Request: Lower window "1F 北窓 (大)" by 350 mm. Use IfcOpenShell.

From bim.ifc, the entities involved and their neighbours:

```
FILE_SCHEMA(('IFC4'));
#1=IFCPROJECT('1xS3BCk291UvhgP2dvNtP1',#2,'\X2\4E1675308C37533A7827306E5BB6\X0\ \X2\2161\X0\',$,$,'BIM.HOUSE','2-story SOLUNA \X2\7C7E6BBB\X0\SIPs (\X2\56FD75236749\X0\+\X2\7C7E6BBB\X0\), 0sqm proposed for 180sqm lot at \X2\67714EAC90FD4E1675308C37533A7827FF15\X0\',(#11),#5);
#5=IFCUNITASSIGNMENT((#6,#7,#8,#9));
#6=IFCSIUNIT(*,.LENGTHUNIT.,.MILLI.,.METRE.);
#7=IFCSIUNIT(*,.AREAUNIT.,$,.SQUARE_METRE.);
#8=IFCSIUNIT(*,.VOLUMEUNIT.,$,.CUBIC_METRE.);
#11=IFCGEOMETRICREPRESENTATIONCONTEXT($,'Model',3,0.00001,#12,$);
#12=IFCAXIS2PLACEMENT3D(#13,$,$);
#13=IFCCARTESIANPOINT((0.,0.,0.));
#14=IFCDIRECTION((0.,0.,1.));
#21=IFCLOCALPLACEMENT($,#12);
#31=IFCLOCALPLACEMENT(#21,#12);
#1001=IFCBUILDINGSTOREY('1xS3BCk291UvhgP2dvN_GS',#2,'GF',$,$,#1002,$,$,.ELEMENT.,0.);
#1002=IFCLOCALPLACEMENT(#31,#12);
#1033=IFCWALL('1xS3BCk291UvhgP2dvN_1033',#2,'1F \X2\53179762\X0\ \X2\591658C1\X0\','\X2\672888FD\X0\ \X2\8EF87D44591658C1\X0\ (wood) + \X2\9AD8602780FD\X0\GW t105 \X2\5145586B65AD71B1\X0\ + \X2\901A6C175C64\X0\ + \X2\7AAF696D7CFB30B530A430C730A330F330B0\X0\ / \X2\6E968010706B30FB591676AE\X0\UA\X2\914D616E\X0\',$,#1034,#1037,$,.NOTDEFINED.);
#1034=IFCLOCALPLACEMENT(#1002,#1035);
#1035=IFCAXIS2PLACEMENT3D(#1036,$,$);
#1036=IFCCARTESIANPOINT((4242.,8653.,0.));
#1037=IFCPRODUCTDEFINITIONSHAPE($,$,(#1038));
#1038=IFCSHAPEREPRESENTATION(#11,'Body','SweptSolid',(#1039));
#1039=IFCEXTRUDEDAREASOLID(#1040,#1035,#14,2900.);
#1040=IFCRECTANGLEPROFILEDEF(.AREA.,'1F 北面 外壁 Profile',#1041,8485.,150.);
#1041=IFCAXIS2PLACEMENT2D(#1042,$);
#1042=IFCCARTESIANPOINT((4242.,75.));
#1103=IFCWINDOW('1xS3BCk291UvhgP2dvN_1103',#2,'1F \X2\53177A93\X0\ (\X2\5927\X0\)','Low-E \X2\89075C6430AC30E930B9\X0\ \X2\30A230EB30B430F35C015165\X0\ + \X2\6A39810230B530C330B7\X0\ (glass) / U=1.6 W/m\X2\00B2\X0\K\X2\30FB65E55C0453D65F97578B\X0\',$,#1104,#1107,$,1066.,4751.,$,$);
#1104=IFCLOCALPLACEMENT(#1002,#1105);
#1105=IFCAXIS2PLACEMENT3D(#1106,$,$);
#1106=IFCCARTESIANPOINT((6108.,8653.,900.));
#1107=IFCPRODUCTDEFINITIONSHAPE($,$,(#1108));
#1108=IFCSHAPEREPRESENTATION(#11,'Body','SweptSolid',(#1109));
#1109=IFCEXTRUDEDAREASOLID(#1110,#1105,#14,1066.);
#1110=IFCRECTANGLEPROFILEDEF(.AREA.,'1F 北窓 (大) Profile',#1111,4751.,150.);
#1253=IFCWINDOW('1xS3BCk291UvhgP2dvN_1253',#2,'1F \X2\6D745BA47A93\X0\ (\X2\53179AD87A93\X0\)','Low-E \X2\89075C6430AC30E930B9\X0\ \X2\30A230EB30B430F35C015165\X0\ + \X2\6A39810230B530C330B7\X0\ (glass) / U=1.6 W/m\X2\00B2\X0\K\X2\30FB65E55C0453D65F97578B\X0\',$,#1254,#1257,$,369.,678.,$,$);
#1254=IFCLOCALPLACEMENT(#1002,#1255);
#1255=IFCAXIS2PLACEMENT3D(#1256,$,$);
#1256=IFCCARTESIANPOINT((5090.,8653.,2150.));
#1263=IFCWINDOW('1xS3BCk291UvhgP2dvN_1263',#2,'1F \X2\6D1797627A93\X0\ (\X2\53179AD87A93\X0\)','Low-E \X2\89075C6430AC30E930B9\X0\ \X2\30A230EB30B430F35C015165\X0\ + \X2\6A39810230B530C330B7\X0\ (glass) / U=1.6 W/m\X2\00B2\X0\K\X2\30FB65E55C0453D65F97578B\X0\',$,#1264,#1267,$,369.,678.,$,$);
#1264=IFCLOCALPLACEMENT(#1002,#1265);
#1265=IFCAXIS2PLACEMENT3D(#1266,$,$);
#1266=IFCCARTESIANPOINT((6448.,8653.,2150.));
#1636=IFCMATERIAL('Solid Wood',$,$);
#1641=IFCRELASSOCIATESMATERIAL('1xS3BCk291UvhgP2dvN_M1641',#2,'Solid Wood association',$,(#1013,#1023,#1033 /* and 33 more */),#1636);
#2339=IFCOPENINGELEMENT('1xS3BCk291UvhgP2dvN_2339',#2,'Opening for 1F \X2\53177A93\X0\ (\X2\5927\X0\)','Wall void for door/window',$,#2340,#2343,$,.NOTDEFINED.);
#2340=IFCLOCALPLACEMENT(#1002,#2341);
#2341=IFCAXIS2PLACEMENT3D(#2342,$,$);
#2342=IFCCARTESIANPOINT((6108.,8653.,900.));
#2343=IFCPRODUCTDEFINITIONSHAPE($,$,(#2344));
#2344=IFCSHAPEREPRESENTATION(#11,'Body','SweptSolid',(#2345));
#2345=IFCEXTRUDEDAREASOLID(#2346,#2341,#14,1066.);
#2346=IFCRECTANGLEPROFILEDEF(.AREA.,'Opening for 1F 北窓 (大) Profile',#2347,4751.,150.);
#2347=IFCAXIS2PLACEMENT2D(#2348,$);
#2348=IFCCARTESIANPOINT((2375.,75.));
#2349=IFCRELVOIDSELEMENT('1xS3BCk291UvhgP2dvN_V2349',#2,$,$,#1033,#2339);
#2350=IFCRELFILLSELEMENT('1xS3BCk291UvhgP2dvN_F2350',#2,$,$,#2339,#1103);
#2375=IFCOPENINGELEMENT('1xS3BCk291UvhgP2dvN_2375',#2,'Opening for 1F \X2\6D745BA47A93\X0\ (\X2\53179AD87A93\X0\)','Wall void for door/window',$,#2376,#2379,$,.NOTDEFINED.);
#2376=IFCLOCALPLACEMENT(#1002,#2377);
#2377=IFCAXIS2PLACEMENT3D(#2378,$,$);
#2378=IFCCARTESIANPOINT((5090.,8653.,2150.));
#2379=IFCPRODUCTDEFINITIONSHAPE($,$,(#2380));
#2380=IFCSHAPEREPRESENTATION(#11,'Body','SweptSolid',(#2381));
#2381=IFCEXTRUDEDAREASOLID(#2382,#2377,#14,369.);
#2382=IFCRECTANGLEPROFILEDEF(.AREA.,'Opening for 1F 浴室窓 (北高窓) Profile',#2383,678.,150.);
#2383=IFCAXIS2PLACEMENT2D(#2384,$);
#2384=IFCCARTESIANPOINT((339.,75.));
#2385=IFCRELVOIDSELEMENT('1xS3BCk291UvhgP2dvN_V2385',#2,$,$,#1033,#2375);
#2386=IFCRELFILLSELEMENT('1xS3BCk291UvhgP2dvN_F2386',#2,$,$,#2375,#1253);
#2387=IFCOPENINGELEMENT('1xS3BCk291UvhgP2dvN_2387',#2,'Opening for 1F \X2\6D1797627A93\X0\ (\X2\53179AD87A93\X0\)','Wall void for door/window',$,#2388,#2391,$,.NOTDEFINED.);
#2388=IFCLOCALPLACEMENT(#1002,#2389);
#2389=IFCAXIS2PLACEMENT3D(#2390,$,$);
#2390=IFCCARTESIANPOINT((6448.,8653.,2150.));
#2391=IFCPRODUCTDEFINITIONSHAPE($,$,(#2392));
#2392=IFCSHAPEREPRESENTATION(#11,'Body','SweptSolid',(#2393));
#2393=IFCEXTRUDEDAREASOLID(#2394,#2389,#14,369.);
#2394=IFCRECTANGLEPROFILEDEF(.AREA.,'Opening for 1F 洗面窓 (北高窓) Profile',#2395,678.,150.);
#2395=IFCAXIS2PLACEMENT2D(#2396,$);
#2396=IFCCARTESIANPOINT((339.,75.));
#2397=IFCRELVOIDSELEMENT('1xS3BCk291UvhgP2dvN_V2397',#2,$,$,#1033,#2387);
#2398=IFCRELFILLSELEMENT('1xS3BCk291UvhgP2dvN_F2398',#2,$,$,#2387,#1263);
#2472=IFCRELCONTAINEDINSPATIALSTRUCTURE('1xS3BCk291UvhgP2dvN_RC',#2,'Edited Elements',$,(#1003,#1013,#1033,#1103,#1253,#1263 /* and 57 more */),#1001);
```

```python
import numpy as np
import ifcopenshell
import ifcopenshell.api.geometry
import ifcopenshell.util.placement
import ifcopenshell.util.unit

model = ifcopenshell.open("bim.ifc")
unit_scale = ifcopenshell.util.unit.calculate_unit_scale(model)

window = model.by_id(1103)
opening = window.FillsVoids[0].RelatingOpeningElement
dz = -0.35 / unit_scale

shift = np.array([0.0, 0.0, dz])
# The window is not placed relative to its opening, so move both.
for product in (opening, window):
    matrix = ifcopenshell.util.placement.get_local_placement(product.ObjectPlacement)
    matrix[:3, 3] += shift
    ifcopenshell.api.geometry.edit_object_placement(model, product=product, matrix=matrix, is_si=False)

print(f"moved by {dz * unit_scale:+.3f} m")

model.write("bim_rev.ifc")
```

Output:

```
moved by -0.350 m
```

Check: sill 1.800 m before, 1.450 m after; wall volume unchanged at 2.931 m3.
